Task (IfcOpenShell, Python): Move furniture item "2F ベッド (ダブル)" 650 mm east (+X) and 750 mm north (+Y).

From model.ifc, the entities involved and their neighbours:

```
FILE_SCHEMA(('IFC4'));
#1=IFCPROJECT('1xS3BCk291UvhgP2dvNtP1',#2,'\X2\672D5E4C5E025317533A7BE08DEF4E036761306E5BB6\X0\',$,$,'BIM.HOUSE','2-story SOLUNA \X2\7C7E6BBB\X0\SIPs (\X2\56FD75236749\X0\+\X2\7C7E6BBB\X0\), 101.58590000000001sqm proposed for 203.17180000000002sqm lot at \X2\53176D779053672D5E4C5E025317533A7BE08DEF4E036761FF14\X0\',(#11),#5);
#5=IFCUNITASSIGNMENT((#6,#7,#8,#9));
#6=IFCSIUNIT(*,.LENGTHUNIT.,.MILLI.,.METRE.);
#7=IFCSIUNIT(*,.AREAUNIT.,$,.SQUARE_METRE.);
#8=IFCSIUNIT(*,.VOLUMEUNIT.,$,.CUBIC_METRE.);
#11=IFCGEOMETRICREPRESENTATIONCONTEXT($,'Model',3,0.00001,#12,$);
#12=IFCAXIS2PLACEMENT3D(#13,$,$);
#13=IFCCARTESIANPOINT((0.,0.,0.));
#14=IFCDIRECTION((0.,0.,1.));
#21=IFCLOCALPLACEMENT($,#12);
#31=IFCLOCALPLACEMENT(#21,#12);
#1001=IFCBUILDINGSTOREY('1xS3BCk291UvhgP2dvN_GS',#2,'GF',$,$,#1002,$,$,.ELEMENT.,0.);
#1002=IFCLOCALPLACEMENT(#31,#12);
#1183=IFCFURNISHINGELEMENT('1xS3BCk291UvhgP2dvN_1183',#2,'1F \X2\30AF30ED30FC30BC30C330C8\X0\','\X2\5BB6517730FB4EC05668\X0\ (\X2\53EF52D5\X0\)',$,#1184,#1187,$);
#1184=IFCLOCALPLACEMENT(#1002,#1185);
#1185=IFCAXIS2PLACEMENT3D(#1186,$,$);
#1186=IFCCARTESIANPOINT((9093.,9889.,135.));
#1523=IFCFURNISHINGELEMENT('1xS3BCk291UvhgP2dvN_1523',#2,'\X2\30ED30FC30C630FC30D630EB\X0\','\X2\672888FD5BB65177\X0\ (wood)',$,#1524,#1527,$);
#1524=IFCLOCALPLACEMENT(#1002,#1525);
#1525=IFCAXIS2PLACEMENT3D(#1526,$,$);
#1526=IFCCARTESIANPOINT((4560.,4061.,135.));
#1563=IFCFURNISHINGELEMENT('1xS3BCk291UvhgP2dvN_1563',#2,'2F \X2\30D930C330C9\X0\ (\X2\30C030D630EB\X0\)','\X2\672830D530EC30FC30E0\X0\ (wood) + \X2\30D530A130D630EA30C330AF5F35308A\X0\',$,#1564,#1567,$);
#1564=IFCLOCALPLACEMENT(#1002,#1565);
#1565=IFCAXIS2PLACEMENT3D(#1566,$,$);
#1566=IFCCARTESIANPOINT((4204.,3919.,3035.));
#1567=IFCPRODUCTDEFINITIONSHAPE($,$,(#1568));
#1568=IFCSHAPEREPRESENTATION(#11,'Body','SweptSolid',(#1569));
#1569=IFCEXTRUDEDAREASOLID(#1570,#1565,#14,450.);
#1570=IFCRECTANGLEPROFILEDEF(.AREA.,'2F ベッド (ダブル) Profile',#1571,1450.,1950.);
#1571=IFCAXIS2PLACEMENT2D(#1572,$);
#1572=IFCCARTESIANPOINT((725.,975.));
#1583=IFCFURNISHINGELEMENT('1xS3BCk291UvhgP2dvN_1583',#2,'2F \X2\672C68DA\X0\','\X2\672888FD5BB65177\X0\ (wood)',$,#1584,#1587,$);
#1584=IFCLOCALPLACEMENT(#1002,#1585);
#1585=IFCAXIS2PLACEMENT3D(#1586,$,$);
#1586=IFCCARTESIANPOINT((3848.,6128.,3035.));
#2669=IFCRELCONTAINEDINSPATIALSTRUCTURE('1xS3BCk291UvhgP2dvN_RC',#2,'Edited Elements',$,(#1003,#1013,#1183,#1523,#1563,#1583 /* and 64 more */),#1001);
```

```python
import ifcopenshell
import ifcopenshell.api.geometry
import ifcopenshell.util.placement

model = ifcopenshell.open("model.ifc")

item = model.by_guid("1xS3BCk291UvhgP2dvN_1563")
matrix = ifcopenshell.util.placement.get_local_placement(item.ObjectPlacement)
matrix[0, 3] += 650.0
matrix[1, 3] += 750.0
ifcopenshell.api.geometry.edit_object_placement(model, product=item, matrix=matrix, is_si=False)

print(ifcopenshell.util.placement.get_local_placement(item.ObjectPlacement).round(3) + 0.0)

model.write("model_v2.ifc")
```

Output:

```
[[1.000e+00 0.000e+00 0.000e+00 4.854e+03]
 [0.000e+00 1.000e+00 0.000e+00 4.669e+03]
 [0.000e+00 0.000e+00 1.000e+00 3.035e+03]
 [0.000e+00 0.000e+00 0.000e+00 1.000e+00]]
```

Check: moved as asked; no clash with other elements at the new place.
